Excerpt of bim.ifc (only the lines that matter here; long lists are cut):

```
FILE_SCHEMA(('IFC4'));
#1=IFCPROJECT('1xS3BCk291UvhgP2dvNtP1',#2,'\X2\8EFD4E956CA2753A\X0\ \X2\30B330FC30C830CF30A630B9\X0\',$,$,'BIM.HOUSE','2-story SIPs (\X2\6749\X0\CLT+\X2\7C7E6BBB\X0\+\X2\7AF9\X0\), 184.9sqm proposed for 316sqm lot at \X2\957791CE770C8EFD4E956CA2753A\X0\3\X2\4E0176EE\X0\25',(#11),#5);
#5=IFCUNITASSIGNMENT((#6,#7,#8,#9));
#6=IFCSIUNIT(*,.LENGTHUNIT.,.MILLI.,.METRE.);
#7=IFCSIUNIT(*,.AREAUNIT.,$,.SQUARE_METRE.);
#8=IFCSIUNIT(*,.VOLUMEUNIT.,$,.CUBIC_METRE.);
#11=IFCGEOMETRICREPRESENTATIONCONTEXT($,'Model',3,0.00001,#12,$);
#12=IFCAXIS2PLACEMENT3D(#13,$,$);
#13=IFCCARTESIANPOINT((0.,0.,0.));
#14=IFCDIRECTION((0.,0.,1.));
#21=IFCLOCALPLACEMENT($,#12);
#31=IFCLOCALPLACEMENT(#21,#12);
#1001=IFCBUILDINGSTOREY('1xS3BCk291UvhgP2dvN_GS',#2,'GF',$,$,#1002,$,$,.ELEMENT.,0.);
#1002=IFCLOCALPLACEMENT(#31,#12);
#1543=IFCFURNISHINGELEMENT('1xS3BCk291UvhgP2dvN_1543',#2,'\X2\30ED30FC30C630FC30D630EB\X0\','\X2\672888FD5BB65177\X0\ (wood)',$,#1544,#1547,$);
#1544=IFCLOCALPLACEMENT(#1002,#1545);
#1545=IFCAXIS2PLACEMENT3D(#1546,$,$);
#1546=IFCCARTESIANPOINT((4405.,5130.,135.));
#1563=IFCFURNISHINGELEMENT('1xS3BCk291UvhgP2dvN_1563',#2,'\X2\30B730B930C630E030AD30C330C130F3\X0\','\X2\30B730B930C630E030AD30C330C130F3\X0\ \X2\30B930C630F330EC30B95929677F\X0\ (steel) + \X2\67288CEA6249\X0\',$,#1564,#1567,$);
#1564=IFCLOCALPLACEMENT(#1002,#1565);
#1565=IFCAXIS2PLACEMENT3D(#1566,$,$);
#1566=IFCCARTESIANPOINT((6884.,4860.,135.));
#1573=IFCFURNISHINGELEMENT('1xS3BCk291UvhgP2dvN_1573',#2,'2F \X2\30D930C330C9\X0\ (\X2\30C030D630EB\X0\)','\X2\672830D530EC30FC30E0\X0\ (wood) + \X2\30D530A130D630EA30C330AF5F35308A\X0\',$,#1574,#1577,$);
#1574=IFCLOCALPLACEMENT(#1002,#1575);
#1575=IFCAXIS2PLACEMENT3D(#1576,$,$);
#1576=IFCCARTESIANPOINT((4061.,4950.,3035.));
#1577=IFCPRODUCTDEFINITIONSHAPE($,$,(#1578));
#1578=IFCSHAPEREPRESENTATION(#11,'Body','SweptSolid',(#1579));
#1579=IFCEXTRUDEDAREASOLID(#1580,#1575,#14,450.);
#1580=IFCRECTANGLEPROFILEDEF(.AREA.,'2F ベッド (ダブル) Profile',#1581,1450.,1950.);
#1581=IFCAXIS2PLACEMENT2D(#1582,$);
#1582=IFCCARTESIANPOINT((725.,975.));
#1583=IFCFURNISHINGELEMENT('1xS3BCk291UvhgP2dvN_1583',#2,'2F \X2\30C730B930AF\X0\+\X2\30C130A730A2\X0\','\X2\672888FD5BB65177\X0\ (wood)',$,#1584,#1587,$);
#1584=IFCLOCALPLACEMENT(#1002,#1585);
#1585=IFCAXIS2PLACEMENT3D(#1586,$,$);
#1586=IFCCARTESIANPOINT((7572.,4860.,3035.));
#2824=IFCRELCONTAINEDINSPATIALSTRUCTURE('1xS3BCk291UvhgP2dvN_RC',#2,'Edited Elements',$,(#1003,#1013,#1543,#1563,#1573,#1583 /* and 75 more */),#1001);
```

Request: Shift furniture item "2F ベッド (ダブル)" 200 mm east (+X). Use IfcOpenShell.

```python
import ifcopenshell
import ifcopenshell.api.geometry
import ifcopenshell.util.placement
import ifcopenshell.util.unit

model = ifcopenshell.open("bim.ifc")
unit_scale = ifcopenshell.util.unit.calculate_unit_scale(model)

item = model.by_guid("1xS3BCk291UvhgP2dvN_1573")
matrix = ifcopenshell.util.placement.get_local_placement(item.ObjectPlacement)
matrix[0, 3] += 0.2 / unit_scale
ifcopenshell.api.geometry.edit_object_placement(model, product=item, matrix=matrix, is_si=False)

print(ifcopenshell.util.placement.get_local_placement(item.ObjectPlacement).round(3) + 0.0)

model.write("bim_rev.ifc")
```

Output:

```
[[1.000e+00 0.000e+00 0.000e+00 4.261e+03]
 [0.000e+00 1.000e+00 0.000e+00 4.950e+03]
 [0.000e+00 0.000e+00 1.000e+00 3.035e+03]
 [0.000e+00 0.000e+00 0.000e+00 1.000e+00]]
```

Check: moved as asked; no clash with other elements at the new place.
